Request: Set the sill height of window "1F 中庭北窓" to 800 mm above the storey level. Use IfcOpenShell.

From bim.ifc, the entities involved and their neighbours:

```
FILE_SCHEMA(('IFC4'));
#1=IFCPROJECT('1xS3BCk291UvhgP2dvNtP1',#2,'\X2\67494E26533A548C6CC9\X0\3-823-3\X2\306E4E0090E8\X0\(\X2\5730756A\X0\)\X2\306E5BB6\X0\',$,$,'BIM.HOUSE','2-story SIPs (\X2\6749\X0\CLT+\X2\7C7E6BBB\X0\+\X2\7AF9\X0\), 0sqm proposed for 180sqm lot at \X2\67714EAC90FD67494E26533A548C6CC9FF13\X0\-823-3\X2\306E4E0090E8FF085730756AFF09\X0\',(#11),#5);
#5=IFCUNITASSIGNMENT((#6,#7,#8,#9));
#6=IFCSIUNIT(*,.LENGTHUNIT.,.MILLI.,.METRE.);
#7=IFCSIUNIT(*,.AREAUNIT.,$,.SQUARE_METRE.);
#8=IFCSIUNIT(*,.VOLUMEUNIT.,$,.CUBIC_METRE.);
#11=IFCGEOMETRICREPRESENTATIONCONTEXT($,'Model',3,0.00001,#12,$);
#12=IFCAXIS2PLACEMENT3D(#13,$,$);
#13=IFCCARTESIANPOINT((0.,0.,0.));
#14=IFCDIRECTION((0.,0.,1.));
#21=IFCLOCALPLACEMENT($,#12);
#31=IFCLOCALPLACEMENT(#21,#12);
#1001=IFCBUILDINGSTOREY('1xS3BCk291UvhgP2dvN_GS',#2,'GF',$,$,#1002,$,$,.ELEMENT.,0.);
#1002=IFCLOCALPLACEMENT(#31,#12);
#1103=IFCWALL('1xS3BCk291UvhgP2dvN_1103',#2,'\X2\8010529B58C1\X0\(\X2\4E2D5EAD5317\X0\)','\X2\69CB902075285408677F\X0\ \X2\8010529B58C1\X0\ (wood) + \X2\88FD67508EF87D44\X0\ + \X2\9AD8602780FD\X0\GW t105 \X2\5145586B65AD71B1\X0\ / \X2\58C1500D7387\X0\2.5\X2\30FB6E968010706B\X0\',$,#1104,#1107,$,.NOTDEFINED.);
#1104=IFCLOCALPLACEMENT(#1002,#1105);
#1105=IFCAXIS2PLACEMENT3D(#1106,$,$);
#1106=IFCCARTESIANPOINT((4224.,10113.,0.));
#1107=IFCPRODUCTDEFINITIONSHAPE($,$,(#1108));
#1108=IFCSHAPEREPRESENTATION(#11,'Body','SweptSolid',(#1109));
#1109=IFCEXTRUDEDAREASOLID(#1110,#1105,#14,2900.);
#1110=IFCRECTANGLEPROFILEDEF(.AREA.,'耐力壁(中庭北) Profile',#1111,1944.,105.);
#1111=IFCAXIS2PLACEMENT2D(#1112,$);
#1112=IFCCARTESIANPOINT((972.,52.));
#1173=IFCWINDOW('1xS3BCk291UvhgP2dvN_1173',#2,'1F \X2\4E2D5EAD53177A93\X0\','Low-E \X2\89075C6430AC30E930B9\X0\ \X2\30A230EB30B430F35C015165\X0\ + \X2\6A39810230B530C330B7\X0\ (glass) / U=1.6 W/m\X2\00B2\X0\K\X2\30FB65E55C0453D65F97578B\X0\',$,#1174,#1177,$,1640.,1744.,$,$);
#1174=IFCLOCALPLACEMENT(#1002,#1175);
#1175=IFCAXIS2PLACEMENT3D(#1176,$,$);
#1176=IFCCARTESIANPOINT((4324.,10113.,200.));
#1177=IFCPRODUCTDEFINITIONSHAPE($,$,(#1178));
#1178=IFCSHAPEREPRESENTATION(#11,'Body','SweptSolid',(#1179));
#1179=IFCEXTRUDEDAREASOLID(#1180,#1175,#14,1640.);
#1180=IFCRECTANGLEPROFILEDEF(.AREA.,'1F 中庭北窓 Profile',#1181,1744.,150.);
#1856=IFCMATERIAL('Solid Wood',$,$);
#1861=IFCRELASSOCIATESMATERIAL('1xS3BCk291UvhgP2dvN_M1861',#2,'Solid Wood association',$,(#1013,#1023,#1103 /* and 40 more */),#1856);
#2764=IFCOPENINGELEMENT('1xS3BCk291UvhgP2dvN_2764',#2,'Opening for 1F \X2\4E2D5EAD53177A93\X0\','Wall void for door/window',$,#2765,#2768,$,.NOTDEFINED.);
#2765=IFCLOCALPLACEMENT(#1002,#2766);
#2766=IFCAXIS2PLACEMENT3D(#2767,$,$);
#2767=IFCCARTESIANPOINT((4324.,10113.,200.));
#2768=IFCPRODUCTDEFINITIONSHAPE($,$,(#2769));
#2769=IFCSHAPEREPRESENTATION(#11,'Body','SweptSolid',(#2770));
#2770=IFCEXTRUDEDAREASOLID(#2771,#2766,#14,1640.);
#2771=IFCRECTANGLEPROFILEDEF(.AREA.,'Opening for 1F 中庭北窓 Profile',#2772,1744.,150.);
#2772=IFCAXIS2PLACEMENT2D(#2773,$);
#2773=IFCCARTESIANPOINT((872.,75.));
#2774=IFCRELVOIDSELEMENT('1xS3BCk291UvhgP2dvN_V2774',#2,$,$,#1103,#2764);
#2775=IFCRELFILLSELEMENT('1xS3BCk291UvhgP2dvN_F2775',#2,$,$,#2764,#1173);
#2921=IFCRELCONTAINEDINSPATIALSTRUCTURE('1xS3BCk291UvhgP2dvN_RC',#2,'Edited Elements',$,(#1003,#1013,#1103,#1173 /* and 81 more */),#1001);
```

```python
import numpy as np
import ifcopenshell
import ifcopenshell.api.geometry
import ifcopenshell.geom
import ifcopenshell.util.element
import ifcopenshell.util.placement
import ifcopenshell.util.shape
import ifcopenshell.util.unit

model = ifcopenshell.open("bim.ifc")
unit_scale = ifcopenshell.util.unit.calculate_unit_scale(model)

window = model.by_guid("1xS3BCk291UvhgP2dvN_1173")
opening = window.FillsVoids[0].RelatingOpeningElement
storey = ifcopenshell.util.element.get_container(window, ifc_class="IfcBuildingStorey")
level = ifcopenshell.util.placement.get_local_placement(storey.ObjectPlacement)[2, 3]

# The opening's origin need not be at the sill, so measure its lowest point.
shape = ifcopenshell.geom.create_shape(ifcopenshell.geom.settings(), opening)
bottom = ifcopenshell.util.shape.get_shape_bottom_elevation(shape, shape.geometry) / unit_scale
dz = level + 800.0 - bottom

shift = np.array([0.0, 0.0, dz])
# The window is not placed relative to its opening, so move both.
for product in (opening, window):
    matrix = ifcopenshell.util.placement.get_local_placement(product.ObjectPlacement)
    matrix[:3, 3] += shift
    ifcopenshell.api.geometry.edit_object_placement(model, product=product, matrix=matrix, is_si=False)

print(f"moved by {dz * unit_scale:+.3f} m")

model.write("bim_edited.ifc")
```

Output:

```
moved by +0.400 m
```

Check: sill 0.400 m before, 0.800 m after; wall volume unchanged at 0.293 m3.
